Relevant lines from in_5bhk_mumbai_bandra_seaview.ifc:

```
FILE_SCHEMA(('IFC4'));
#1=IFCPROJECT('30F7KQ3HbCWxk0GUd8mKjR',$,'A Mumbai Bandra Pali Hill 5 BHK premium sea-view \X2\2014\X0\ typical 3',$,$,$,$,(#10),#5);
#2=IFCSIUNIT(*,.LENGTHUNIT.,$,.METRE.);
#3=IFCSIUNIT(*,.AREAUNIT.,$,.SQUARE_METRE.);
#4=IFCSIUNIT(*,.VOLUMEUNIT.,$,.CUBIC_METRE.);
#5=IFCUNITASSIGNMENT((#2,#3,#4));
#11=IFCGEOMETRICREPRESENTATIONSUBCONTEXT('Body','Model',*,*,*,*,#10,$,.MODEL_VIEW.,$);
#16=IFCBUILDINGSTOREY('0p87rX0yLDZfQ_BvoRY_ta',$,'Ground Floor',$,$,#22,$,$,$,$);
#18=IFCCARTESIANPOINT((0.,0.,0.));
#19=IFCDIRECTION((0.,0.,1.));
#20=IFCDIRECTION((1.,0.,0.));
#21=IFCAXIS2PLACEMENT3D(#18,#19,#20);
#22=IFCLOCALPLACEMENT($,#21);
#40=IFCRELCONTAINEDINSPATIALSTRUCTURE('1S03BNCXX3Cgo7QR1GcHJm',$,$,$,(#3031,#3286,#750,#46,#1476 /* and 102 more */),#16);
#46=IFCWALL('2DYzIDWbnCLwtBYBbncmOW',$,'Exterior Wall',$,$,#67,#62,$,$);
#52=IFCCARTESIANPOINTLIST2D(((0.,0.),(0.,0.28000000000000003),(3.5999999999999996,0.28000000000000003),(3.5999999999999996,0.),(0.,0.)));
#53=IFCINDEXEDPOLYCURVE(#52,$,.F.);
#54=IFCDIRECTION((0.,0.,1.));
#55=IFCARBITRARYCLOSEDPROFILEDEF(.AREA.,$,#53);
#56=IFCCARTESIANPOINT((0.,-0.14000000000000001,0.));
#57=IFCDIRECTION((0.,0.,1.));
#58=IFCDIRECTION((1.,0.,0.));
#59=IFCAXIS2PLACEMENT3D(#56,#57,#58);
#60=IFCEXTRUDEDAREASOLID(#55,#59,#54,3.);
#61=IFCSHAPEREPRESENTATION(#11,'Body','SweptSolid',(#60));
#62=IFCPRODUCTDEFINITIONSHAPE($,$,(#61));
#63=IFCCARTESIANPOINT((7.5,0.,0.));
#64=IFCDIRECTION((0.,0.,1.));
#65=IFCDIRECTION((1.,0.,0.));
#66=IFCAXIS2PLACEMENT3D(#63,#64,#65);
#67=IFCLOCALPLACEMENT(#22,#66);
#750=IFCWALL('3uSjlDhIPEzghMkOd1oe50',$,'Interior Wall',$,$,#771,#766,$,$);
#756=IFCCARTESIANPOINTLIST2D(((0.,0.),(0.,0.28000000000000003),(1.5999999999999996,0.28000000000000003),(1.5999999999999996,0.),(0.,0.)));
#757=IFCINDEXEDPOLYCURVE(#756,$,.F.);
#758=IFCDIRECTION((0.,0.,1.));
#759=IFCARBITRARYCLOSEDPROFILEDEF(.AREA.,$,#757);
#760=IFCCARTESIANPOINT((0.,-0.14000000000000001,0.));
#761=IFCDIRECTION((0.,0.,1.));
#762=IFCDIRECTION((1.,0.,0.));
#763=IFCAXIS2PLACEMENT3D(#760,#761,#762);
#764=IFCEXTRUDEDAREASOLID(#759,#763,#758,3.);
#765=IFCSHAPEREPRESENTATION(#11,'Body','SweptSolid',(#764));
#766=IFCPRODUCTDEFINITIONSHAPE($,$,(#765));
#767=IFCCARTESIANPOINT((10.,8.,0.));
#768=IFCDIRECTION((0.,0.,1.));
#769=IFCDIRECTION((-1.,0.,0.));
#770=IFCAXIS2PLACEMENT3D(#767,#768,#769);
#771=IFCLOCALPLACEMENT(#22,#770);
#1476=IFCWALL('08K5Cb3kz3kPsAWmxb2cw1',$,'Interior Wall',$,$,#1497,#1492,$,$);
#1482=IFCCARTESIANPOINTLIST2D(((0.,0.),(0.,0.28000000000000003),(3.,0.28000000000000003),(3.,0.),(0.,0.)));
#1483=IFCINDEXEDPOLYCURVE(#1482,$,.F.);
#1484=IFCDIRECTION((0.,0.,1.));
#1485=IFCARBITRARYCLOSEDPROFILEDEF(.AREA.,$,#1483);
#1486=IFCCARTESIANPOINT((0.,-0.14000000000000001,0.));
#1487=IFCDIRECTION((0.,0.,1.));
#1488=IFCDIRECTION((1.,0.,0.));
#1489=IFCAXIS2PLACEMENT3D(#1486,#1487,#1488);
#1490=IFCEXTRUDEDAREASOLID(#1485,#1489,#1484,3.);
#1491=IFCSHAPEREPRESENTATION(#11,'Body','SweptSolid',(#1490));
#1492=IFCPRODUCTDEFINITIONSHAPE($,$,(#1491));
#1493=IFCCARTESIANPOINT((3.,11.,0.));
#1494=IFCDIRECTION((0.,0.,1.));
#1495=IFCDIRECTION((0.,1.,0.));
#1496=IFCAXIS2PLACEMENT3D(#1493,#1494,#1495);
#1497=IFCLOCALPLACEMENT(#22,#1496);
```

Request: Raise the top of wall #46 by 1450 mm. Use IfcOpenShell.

```python
import ifcopenshell
import ifcopenshell.geom
import ifcopenshell.util.representation
import ifcopenshell.util.shape

model = ifcopenshell.open("in_5bhk_mumbai_bandra_seaview.ifc")
settings = ifcopenshell.geom.settings()


def volume(element):
    """Net volume in cubic metres, openings subtracted."""
    shape = ifcopenshell.geom.create_shape(settings, element)
    return ifcopenshell.util.shape.get_volume(shape.geometry)


wall = model.by_guid("2DYzIDWbnCLwtBYBbncmOW")
before = volume(wall)

body = ifcopenshell.util.representation.get_representation(wall, "Model", "Body")
solid = body.Items[0]
old_height = solid.Depth
solid.Depth += 1.45
after = volume(wall)

print(f"height {old_height:g} -> {solid.Depth:g}, volume {before:.3f} -> {after:.3f} m3")

model.write("in_5bhk_mumbai_bandra_seaview_rev.ifc")
```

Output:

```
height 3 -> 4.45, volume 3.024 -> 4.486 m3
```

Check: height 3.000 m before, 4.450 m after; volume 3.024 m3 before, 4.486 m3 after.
